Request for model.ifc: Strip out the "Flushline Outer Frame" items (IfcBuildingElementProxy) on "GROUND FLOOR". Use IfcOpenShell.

First a look at what the model holds.

```python
import ifcopenshell
import ifcopenshell.util.element

model = ifcopenshell.open("model.ifc")
print(model.schema)
storey = next(s for s in model.by_type("IfcBuildingStorey") if s.Name == "GROUND FLOOR")
proxies = [e for e in ifcopenshell.util.element.get_decomposition(storey) if e.is_a("IfcBuildingElementProxy")]
seen = {}
for e in proxies:
    element_type = ifcopenshell.util.element.get_type(e)
    name = element_type.Name if element_type not in (None, e) else None
    seen[name] = seen.get(name, 0) + 1
for name, count in sorted(seen.items(), key=str):
    print(count, "x", name)
```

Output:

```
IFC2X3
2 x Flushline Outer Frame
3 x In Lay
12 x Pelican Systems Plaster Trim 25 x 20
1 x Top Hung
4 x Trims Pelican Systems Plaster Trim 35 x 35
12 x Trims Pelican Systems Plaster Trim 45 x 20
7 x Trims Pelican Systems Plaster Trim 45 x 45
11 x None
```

```python
import ifcopenshell
import ifcopenshell.api.root
import ifcopenshell.util.element

model = ifcopenshell.open("model.ifc")

storey = next(s for s in model.by_type("IfcBuildingStorey") if s.Name == "GROUND FLOOR")
proxies = [e for e in ifcopenshell.util.element.get_decomposition(storey) if e.is_a("IfcBuildingElementProxy")]
targets = [e for e in proxies if (t := ifcopenshell.util.element.get_type(e)) not in (None, e) and t.Name == "Flushline Outer Frame"]

for e in targets:
    ifcopenshell.api.root.remove_product(model, product=e)
print(len(targets), "removed")

model.write("model_v2.ifc")
```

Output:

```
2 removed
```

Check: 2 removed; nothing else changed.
